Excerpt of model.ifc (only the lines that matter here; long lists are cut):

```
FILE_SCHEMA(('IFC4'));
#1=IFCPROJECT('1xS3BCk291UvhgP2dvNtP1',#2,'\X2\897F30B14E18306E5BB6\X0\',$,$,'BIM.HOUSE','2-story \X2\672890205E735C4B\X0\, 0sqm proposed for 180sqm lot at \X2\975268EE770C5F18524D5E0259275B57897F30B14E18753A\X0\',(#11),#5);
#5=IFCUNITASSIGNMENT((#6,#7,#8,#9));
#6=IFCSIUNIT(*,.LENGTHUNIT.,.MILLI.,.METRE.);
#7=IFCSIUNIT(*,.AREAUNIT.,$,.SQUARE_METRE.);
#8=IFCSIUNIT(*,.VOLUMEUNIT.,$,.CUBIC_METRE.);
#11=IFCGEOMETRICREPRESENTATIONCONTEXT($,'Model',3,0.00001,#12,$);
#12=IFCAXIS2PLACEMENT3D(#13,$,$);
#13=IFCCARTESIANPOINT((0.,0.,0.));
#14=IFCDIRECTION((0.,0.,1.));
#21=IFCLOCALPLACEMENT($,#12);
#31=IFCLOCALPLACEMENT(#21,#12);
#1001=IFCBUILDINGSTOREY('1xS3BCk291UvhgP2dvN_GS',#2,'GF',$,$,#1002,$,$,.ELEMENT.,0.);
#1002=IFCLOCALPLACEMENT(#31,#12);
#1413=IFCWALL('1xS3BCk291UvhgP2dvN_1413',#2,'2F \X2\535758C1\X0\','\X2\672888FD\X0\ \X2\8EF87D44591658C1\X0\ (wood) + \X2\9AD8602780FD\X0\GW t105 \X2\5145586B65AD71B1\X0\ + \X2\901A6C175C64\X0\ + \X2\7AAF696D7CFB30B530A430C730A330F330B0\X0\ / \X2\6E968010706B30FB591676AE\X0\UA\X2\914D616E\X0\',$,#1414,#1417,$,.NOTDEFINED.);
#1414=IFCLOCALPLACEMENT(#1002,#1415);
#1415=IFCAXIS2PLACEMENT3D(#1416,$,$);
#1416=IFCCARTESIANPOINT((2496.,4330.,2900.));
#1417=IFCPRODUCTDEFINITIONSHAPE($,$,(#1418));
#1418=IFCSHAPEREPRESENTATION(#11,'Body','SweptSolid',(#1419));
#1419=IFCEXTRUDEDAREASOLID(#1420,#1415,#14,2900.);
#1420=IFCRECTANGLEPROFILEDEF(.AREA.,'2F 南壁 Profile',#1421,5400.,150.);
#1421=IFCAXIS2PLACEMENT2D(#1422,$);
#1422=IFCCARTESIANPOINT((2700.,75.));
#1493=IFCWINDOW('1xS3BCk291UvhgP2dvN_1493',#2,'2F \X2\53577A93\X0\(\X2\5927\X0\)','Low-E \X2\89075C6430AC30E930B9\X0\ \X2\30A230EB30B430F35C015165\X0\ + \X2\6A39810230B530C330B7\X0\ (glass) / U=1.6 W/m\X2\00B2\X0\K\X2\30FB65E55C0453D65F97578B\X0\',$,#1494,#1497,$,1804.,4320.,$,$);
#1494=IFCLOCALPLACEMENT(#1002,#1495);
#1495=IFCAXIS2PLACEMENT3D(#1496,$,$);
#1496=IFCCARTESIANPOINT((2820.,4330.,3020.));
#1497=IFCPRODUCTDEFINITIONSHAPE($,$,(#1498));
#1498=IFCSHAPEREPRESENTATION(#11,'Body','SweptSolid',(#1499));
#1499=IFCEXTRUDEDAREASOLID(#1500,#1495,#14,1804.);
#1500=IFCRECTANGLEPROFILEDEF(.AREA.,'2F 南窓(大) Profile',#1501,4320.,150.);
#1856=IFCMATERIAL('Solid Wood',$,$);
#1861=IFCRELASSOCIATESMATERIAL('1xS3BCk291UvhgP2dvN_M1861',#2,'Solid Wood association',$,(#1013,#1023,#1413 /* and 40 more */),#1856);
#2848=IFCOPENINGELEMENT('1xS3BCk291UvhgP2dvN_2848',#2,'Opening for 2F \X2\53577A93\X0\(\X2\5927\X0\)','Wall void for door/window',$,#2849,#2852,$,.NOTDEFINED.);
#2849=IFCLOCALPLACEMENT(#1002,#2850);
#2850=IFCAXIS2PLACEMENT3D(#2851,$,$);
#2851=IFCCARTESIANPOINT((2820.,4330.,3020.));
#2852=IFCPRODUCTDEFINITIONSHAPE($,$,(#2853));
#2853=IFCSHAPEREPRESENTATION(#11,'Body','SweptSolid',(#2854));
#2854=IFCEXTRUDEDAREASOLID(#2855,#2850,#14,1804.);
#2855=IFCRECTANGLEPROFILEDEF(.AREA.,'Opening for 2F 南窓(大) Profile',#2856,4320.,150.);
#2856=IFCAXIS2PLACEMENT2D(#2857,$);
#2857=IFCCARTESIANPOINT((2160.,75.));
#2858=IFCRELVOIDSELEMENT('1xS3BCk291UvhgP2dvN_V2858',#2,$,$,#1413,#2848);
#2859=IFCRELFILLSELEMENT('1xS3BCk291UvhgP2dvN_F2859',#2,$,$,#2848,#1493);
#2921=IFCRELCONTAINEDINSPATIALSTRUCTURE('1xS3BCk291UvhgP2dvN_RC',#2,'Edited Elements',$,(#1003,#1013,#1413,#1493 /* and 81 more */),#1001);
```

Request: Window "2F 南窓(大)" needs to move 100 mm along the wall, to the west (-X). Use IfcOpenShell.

```python
import ifcopenshell
import ifcopenshell.api.geometry
import ifcopenshell.util.placement
import ifcopenshell.util.unit

model = ifcopenshell.open("model.ifc")
unit_scale = ifcopenshell.util.unit.calculate_unit_scale(model)

window = model.by_guid("1xS3BCk291UvhgP2dvN_1493")
opening = window.FillsVoids[0].RelatingOpeningElement
wall = opening.VoidsElements[0].RelatingBuildingElement

wall_matrix = ifcopenshell.util.placement.get_local_placement(wall.ObjectPlacement)
shift = wall_matrix[:3, 0] * -0.1 / unit_scale
before = ifcopenshell.util.placement.get_local_placement(window.ObjectPlacement)[:3, 3].copy()

# The window is not placed relative to its opening, so move both.
for product in (opening, window):
    matrix = ifcopenshell.util.placement.get_local_placement(product.ObjectPlacement)
    matrix[:3, 3] += shift
    ifcopenshell.api.geometry.edit_object_placement(model, product=product, matrix=matrix, is_si=False)

after = ifcopenshell.util.placement.get_local_placement(window.ObjectPlacement)[:3, 3]
print("window moved by", (after - before).round(3) + 0.0)

model.write("model_v2.ifc")
```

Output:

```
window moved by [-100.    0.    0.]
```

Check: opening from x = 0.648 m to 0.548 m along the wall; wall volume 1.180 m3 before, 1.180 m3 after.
